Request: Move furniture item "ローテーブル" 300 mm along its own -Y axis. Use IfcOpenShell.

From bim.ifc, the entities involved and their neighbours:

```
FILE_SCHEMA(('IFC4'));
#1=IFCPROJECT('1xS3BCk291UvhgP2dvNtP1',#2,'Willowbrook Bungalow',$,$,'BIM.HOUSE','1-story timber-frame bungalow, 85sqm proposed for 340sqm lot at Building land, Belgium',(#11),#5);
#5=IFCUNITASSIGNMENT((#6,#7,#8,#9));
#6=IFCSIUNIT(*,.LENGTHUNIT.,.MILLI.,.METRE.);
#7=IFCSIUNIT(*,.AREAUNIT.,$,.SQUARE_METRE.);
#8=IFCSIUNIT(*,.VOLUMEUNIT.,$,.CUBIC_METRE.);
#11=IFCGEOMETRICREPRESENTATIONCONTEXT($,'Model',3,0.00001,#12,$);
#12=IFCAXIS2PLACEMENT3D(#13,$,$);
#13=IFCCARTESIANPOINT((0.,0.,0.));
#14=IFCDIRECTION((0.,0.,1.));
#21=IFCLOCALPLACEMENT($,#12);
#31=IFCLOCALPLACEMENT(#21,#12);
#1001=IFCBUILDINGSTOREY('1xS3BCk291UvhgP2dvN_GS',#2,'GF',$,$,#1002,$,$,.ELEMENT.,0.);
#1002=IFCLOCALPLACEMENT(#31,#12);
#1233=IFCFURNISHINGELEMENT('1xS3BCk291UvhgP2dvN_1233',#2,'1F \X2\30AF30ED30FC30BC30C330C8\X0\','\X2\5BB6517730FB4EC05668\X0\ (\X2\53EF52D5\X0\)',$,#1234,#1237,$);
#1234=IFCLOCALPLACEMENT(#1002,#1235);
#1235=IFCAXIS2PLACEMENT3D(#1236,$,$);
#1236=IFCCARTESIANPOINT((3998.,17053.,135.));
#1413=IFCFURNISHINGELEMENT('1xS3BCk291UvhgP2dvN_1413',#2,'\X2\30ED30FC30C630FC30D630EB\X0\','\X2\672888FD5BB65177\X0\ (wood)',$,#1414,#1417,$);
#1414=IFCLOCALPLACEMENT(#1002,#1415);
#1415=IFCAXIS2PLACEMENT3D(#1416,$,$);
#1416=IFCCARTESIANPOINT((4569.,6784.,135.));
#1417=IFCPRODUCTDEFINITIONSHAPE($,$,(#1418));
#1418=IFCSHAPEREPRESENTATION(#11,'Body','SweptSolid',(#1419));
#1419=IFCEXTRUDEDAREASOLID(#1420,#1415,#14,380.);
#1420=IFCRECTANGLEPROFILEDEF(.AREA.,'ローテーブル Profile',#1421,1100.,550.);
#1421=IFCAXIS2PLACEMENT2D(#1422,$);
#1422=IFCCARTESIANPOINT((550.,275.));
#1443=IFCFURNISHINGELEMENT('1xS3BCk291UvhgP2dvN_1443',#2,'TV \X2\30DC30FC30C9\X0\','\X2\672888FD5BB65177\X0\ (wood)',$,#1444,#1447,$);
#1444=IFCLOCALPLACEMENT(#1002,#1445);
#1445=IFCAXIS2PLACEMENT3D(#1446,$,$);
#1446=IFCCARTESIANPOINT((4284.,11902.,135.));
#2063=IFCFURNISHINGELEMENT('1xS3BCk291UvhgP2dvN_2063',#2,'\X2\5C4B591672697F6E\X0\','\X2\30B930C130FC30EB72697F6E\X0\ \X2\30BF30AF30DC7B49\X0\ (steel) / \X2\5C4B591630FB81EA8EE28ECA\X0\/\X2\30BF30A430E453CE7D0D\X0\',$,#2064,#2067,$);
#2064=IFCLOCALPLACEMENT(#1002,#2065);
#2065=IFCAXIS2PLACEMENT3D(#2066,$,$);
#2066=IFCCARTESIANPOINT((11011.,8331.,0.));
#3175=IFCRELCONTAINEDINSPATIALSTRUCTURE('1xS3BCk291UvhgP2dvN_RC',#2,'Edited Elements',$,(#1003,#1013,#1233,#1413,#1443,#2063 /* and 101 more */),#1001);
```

```python
import ifcopenshell
import ifcopenshell.api.geometry
import ifcopenshell.util.placement
import ifcopenshell.util.unit

model = ifcopenshell.open("bim.ifc")
unit_scale = ifcopenshell.util.unit.calculate_unit_scale(model)

item = model.by_guid("1xS3BCk291UvhgP2dvN_1413")
matrix = ifcopenshell.util.placement.get_local_placement(item.ObjectPlacement)
matrix[:3, 3] -= matrix[:3, 1] * 0.3 / unit_scale
ifcopenshell.api.geometry.edit_object_placement(model, product=item, matrix=matrix, is_si=False)

print(ifcopenshell.util.placement.get_local_placement(item.ObjectPlacement).round(3) + 0.0)

model.write("bim_edited.ifc")
```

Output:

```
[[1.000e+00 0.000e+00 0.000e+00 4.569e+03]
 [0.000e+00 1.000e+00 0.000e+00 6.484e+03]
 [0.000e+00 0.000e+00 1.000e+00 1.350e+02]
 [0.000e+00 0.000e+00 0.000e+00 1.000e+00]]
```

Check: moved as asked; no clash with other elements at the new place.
